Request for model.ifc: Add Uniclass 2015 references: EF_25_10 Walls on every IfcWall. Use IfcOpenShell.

First a look at what the model holds.

```python
import ifcopenshell

model = ifcopenshell.open("model.ifc")
print(model.schema)
print("classifications:", [c.Name for c in model.by_type("IfcClassification")])
for ifc_class in ("IfcDoor", "IfcRoof", "IfcStair", "IfcWall", "IfcWindow"):
    print(ifc_class, len(model.by_type(ifc_class)))
```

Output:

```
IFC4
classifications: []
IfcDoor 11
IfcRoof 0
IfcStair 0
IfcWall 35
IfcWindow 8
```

```python
import ifcopenshell
import ifcopenshell.api.classification

model = ifcopenshell.open("model.ifc")

system = ifcopenshell.api.classification.add_classification(model, classification="Uniclass 2015")

codes = {
    "IfcWall": ("EF_25_10", "Walls"),
}
for ifc_class, (code, name) in codes.items():
    products = model.by_type(ifc_class)
    ifcopenshell.api.classification.add_reference(
        model, products=products, classification=system, identification=code, name=name
    )
    print(code, len(products))

model.write("model_updated.ifc")
```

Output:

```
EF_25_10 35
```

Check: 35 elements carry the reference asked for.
